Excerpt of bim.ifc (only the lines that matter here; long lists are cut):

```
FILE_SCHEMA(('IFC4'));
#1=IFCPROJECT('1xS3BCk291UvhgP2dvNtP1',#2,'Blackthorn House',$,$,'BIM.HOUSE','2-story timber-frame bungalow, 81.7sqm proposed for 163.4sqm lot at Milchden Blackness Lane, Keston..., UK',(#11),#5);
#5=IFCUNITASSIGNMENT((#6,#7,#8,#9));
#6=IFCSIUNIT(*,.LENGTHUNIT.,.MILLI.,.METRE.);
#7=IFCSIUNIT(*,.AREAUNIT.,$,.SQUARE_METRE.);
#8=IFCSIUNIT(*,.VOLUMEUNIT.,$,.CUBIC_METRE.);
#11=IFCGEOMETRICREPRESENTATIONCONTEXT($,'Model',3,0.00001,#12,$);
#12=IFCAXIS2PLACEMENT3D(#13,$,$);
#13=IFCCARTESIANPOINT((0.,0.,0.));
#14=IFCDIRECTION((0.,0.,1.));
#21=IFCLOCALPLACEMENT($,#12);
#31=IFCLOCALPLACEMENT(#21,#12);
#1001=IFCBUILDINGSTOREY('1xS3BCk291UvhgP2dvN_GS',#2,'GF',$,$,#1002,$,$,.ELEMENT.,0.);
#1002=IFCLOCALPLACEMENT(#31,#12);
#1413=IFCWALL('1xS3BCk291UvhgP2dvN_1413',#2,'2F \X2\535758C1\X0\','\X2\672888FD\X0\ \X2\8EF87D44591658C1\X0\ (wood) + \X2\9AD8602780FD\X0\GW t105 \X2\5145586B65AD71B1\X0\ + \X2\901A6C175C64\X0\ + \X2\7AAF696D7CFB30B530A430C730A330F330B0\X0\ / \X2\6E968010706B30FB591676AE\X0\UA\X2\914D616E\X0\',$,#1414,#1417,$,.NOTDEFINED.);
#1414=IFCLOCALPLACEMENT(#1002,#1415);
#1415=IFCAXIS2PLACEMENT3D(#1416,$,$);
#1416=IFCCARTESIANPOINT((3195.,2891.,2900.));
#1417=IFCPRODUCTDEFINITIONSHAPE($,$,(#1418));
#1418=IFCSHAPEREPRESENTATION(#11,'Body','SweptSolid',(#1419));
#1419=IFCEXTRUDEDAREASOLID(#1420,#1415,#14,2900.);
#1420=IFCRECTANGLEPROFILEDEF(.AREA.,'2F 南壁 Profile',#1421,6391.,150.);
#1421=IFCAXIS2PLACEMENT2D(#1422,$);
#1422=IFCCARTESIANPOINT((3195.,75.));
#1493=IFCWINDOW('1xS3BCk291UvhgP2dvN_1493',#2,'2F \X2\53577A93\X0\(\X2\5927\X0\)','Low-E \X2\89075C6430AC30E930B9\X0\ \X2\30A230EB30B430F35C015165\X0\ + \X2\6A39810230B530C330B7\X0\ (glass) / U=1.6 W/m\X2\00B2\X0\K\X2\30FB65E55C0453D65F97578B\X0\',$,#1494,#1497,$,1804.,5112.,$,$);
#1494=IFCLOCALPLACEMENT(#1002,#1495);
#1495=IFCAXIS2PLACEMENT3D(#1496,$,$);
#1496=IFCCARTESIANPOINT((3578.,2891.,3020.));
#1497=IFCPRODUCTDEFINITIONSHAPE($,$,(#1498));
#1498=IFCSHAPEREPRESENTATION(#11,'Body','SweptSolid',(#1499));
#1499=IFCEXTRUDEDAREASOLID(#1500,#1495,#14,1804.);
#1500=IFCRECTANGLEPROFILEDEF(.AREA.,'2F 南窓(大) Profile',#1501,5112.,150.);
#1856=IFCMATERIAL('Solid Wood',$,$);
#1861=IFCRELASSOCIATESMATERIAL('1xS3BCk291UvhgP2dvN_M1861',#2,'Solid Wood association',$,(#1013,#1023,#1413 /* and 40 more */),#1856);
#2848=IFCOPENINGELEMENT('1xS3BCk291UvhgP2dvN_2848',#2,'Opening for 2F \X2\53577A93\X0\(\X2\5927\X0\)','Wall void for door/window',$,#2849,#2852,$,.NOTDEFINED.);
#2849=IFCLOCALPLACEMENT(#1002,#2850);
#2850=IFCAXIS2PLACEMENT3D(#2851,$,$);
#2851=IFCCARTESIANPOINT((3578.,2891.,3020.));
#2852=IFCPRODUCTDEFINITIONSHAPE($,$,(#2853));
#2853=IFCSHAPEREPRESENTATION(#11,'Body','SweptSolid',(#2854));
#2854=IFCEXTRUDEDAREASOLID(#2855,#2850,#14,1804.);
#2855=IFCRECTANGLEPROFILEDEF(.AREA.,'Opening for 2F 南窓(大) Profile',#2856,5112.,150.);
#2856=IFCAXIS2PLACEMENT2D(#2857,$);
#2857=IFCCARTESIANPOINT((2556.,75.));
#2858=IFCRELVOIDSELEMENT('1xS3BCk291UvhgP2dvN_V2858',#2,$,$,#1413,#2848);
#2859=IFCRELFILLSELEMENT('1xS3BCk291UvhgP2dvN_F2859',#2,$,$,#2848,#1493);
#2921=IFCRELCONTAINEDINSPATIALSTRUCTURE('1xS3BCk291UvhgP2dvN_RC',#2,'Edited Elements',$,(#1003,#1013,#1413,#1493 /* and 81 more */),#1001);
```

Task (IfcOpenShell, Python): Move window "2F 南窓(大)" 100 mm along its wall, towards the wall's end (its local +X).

```python
import ifcopenshell
import ifcopenshell.api.geometry
import ifcopenshell.util.placement
import ifcopenshell.util.unit

model = ifcopenshell.open("bim.ifc")
unit_scale = ifcopenshell.util.unit.calculate_unit_scale(model)

window = model.by_id(1493)
opening = window.FillsVoids[0].RelatingOpeningElement
wall = opening.VoidsElements[0].RelatingBuildingElement

wall_matrix = ifcopenshell.util.placement.get_local_placement(wall.ObjectPlacement)
shift = wall_matrix[:3, 0] * 0.1 / unit_scale
before = ifcopenshell.util.placement.get_local_placement(window.ObjectPlacement)[:3, 3].copy()

# The window is not placed relative to its opening, so move both.
for product in (opening, window):
    matrix = ifcopenshell.util.placement.get_local_placement(product.ObjectPlacement)
    matrix[:3, 3] += shift
    ifcopenshell.api.geometry.edit_object_placement(model, product=product, matrix=matrix, is_si=False)

after = ifcopenshell.util.placement.get_local_placement(window.ObjectPlacement)[:3, 3]
print("window moved by", (after - before).round(3) + 0.0)

model.write("bim_edited.ifc")
```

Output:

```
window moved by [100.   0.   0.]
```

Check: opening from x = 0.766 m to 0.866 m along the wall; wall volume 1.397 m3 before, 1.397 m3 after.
